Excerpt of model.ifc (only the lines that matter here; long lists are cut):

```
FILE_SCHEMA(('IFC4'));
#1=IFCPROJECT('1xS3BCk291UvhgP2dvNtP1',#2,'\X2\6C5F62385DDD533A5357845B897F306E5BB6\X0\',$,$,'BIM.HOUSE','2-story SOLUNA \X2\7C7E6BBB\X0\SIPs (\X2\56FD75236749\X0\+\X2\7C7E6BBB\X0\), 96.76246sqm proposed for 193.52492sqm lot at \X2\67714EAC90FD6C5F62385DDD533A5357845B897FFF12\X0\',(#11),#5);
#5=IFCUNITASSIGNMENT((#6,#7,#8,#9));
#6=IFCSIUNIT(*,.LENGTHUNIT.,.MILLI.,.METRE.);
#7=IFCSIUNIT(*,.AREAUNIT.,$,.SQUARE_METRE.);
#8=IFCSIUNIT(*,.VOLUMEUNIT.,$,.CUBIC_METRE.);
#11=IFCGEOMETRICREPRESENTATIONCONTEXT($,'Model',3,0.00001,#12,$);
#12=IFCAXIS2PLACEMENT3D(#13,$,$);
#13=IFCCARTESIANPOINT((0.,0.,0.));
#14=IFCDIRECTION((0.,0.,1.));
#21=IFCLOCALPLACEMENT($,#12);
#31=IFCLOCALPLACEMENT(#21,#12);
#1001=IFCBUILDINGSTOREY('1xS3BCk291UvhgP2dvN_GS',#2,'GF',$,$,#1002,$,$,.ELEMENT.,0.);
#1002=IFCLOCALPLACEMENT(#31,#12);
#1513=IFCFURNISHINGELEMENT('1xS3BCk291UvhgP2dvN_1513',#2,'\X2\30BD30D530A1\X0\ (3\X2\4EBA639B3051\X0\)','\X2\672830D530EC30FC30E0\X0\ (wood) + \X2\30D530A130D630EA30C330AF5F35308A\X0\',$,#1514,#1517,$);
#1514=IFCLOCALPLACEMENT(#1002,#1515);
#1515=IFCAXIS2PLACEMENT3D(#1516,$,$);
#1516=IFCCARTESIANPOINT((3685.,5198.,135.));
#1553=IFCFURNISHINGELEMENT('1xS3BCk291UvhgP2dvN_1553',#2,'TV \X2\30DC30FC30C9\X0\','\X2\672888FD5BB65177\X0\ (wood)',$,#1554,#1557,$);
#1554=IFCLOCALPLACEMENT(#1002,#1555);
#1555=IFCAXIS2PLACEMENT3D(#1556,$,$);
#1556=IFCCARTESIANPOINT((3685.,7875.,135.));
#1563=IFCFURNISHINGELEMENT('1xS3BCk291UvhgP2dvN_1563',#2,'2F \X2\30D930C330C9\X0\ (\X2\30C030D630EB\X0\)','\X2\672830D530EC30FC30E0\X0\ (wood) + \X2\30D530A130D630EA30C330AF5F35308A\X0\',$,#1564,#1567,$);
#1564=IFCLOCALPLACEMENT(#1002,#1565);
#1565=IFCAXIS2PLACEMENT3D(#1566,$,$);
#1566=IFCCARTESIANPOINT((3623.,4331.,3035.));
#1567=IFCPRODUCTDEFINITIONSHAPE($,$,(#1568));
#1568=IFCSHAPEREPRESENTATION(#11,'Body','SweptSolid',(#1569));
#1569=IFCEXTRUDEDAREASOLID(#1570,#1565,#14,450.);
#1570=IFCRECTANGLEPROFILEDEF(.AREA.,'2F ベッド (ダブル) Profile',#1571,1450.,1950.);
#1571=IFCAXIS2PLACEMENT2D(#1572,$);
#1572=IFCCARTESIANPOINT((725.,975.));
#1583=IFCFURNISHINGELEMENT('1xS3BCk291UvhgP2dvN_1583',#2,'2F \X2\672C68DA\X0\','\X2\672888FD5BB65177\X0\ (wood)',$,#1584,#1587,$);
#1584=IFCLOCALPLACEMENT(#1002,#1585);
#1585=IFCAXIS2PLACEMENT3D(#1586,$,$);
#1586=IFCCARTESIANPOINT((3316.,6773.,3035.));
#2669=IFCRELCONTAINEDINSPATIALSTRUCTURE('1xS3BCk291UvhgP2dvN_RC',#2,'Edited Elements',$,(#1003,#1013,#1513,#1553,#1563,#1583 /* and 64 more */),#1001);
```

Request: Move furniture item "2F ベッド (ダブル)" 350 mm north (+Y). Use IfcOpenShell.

```python
import ifcopenshell
import ifcopenshell.api.geometry
import ifcopenshell.util.placement

model = ifcopenshell.open("model.ifc")

item = model.by_id(1563)
matrix = ifcopenshell.util.placement.get_local_placement(item.ObjectPlacement)
matrix[1, 3] += 350.0
ifcopenshell.api.geometry.edit_object_placement(model, product=item, matrix=matrix, is_si=False)

print(ifcopenshell.util.placement.get_local_placement(item.ObjectPlacement).round(3) + 0.0)

model.write("model_rev.ifc")
```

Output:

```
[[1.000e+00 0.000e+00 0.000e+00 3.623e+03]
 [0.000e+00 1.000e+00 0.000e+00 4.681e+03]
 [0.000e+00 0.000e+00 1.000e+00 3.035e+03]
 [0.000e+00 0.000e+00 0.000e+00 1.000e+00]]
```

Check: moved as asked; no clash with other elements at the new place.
